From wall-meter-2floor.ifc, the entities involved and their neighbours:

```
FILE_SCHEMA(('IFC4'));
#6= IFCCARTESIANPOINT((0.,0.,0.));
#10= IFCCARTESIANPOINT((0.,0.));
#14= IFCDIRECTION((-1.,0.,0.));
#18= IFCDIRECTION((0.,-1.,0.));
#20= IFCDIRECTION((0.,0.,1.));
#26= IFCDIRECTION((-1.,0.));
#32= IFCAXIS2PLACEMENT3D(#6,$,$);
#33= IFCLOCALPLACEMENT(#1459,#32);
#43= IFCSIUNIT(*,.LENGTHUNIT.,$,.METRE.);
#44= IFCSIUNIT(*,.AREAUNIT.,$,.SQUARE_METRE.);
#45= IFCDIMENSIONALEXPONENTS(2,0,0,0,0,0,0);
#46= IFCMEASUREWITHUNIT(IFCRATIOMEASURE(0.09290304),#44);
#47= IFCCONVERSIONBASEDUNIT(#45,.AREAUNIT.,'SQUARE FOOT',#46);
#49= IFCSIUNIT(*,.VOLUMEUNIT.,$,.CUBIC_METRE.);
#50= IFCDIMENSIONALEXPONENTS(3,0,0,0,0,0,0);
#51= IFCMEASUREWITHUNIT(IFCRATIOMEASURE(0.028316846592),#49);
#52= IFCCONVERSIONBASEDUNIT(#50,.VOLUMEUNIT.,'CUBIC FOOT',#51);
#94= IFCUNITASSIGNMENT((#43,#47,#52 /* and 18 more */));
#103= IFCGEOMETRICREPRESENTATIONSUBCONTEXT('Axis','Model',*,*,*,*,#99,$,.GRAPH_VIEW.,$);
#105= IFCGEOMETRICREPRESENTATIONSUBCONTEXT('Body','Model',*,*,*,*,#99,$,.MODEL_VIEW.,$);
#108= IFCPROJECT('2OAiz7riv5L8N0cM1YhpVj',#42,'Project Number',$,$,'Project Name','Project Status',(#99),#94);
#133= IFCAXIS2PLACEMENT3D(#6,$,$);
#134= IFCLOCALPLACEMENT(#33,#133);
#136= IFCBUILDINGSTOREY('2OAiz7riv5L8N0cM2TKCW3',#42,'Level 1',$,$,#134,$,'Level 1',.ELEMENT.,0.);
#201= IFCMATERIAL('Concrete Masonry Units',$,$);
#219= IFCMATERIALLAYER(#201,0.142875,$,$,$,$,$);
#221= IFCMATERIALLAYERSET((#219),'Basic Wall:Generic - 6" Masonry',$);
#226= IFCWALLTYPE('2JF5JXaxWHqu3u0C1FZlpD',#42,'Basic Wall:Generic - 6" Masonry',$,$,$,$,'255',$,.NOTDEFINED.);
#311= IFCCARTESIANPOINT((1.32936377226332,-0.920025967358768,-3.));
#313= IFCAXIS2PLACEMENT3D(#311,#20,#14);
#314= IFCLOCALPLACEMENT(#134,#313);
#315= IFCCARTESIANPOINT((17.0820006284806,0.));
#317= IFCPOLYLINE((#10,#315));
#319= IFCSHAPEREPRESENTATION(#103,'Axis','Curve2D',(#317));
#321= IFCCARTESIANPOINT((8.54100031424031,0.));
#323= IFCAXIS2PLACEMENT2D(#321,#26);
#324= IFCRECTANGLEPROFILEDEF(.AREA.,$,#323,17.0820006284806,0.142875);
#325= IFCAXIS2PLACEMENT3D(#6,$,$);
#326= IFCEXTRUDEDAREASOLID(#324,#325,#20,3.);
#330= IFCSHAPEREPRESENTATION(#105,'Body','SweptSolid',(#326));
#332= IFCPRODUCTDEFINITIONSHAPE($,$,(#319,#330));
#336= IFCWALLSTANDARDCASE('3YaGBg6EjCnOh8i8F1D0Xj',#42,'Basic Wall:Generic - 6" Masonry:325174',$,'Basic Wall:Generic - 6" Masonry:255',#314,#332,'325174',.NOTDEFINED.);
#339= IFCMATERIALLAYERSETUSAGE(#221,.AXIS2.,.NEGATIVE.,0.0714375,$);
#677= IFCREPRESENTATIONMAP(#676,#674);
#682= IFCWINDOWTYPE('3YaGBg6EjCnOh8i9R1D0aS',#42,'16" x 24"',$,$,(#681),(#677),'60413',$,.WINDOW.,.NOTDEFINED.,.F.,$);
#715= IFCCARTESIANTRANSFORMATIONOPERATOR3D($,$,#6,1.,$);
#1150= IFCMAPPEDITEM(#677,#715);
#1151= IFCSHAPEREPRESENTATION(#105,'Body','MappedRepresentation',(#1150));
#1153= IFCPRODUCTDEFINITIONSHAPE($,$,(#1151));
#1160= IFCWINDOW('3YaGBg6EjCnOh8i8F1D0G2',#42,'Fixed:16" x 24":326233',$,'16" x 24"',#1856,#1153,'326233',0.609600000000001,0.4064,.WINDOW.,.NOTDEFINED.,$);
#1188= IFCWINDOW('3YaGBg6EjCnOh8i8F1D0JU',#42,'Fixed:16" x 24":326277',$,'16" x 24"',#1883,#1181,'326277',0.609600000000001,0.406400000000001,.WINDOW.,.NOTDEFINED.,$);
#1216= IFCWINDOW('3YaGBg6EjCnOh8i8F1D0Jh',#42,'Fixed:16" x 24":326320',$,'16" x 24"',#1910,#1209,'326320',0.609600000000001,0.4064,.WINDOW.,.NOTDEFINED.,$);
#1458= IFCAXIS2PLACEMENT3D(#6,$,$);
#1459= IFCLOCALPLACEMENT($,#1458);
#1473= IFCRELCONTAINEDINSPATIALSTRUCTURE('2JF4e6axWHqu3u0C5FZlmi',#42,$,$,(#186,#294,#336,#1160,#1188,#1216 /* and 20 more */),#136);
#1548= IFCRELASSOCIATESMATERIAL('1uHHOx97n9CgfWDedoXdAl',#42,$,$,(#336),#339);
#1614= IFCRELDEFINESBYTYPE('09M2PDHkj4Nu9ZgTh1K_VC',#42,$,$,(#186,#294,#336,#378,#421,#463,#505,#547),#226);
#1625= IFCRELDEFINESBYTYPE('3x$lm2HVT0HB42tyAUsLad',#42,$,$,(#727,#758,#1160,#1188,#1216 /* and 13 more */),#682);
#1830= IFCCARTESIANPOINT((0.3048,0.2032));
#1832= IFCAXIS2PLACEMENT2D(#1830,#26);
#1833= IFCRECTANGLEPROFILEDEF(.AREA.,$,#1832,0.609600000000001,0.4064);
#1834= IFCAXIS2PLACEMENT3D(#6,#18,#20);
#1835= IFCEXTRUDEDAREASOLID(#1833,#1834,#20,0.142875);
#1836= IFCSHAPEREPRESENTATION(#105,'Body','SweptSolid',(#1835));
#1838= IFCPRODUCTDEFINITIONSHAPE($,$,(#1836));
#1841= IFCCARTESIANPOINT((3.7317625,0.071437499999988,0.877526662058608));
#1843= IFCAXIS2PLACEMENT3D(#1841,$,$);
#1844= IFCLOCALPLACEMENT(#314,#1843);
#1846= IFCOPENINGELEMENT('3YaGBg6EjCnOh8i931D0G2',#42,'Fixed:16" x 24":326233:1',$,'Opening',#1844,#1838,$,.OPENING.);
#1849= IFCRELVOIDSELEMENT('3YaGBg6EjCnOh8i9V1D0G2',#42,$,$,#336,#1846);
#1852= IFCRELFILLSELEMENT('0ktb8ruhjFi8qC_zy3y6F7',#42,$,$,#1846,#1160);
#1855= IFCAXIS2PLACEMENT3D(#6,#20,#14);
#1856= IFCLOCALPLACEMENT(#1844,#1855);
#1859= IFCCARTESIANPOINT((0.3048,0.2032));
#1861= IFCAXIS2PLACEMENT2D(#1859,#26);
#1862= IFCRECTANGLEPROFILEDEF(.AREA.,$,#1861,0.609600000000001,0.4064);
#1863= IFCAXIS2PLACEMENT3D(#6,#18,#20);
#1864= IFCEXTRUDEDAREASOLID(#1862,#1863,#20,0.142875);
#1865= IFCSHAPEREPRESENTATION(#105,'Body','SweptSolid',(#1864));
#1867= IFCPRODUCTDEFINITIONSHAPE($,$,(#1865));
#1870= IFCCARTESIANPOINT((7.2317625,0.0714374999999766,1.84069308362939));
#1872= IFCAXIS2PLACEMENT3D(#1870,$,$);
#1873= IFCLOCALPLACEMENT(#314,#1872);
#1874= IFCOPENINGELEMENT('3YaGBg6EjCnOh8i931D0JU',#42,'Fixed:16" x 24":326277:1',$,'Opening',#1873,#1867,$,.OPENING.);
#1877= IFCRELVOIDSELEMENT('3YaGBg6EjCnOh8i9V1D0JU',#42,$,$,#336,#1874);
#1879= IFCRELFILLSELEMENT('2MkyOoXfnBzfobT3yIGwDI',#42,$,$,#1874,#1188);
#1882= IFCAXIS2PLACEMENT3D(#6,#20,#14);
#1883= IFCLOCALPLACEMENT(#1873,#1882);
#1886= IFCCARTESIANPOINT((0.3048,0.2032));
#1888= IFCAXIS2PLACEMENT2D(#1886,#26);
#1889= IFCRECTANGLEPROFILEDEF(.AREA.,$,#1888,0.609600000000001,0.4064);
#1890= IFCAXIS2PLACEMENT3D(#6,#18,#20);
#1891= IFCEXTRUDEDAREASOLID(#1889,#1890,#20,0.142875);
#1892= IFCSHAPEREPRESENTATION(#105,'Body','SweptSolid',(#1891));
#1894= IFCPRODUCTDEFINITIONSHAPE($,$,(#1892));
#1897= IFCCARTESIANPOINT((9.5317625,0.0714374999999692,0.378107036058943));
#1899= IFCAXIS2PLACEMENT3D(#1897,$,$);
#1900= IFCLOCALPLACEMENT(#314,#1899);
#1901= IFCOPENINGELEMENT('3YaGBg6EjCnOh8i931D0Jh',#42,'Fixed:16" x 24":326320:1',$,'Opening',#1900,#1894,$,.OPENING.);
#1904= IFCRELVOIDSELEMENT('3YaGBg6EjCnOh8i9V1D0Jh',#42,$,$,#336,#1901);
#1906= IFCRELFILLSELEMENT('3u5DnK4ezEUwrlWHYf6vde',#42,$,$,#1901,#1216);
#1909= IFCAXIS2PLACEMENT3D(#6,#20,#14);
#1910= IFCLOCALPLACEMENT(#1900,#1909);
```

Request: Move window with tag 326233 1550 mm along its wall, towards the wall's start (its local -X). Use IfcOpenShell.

```python
import ifcopenshell
import ifcopenshell.api.geometry
import ifcopenshell.util.placement
import ifcopenshell.util.unit

model = ifcopenshell.open("wall-meter-2floor.ifc")
unit_scale = ifcopenshell.util.unit.calculate_unit_scale(model)

window = model.by_guid("3YaGBg6EjCnOh8i8F1D0G2")
opening = window.FillsVoids[0].RelatingOpeningElement
wall = opening.VoidsElements[0].RelatingBuildingElement

wall_matrix = ifcopenshell.util.placement.get_local_placement(wall.ObjectPlacement)
shift = wall_matrix[:3, 0] * -1.55 / unit_scale
before = ifcopenshell.util.placement.get_local_placement(window.ObjectPlacement)[:3, 3].copy()

# The window is placed relative to its opening, so it follows when the opening moves.
matrix = ifcopenshell.util.placement.get_local_placement(opening.ObjectPlacement)
matrix[:3, 3] += shift
ifcopenshell.api.geometry.edit_object_placement(
    model, product=opening, matrix=matrix, is_si=False, should_transform_children=True
)

after = ifcopenshell.util.placement.get_local_placement(window.ObjectPlacement)[:3, 3]
print("window moved by", (after - before).round(3) + 0.0)

model.write("wall-meter-2floor_updated.ifc")
```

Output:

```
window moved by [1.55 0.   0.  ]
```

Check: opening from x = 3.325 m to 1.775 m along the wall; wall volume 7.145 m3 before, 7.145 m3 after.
